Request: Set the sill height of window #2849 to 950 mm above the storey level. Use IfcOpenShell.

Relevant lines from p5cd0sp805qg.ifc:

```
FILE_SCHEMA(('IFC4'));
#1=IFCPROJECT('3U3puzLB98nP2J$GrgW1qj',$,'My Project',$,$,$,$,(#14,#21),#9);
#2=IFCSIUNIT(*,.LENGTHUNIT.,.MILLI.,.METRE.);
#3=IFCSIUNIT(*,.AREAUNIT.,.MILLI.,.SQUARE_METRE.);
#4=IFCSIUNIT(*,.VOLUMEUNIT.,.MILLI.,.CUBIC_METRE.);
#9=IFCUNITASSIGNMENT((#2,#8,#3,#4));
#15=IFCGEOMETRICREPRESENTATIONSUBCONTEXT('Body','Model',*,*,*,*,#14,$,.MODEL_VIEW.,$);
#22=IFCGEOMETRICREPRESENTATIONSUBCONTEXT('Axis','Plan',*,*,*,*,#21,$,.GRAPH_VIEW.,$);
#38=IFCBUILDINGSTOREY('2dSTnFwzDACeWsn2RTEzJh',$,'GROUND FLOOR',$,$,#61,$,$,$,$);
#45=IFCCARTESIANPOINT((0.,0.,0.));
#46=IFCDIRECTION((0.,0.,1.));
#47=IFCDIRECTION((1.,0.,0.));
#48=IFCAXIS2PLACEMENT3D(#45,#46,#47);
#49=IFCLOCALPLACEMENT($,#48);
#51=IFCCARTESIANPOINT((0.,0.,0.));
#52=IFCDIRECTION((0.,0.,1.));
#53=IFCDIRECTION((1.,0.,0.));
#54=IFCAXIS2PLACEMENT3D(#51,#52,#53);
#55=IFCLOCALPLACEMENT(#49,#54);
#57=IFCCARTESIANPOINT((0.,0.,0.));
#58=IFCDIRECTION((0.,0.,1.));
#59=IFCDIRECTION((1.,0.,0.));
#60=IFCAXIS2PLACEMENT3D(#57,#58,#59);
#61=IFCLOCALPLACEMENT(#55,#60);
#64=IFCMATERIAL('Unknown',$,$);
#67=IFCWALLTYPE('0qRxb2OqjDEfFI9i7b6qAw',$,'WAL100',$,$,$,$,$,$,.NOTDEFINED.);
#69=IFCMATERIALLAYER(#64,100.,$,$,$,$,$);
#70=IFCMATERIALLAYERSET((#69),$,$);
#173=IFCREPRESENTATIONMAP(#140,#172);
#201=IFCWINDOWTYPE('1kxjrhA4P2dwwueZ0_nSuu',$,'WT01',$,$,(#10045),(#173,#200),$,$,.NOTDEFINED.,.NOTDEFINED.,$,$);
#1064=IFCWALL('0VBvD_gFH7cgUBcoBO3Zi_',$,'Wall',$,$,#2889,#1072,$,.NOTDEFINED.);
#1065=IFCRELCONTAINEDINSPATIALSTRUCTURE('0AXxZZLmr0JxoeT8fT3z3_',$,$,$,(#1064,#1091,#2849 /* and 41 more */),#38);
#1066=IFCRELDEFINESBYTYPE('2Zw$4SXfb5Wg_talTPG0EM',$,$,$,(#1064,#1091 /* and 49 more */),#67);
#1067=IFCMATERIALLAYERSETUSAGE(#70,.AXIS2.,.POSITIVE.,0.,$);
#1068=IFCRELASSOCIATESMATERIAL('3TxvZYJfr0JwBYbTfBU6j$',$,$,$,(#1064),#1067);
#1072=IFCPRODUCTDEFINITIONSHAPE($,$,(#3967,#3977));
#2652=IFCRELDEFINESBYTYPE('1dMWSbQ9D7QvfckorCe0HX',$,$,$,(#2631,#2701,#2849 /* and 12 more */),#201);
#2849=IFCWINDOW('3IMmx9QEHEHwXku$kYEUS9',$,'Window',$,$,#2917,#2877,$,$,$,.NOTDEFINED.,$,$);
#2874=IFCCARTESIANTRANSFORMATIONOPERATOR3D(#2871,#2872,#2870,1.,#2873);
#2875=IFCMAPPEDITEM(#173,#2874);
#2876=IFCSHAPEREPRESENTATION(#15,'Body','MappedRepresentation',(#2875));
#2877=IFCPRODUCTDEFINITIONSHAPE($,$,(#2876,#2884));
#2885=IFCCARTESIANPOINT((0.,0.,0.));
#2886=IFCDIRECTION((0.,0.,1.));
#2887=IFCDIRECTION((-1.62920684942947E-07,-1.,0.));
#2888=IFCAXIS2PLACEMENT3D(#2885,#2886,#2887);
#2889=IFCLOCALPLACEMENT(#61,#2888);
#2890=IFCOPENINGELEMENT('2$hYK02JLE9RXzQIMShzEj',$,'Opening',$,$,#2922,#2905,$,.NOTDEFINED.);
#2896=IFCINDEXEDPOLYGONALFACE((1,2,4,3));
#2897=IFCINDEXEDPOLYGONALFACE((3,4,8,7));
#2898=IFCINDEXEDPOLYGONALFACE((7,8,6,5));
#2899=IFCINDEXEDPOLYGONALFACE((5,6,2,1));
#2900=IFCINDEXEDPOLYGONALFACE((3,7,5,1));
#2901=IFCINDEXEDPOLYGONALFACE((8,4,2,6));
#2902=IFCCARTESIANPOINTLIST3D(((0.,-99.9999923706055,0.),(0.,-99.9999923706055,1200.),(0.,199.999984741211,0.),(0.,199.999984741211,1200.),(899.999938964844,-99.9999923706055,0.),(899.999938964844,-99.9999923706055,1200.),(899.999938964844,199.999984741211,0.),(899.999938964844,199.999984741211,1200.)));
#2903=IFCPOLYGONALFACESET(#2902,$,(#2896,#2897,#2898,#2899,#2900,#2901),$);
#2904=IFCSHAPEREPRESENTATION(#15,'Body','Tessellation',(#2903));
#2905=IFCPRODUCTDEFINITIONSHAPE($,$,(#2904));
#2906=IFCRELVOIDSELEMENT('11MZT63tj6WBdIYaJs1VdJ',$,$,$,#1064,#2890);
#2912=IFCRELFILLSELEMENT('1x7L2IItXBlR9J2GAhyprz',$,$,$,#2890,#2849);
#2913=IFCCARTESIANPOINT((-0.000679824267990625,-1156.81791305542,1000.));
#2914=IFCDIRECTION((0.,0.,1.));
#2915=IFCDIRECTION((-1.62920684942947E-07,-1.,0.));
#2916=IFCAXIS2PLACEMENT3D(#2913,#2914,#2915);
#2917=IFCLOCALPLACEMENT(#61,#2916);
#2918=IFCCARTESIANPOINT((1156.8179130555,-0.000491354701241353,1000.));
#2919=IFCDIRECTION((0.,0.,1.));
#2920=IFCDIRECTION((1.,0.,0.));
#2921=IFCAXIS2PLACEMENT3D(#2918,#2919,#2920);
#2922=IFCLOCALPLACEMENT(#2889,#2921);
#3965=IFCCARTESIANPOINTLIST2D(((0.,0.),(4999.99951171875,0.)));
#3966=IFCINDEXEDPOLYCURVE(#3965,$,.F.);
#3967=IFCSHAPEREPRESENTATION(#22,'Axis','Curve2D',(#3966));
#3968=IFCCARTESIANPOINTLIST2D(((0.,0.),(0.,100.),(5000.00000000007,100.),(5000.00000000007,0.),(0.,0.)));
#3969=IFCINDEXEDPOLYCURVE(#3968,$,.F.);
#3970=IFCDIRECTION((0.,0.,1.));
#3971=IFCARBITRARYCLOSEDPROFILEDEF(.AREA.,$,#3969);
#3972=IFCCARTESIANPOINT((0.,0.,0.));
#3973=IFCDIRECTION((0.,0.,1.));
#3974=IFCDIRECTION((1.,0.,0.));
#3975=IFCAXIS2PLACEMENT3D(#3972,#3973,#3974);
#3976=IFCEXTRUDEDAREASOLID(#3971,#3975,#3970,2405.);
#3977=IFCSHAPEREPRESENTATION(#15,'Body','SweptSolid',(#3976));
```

```python
import numpy as np
import ifcopenshell
import ifcopenshell.api.geometry
import ifcopenshell.geom
import ifcopenshell.util.element
import ifcopenshell.util.placement
import ifcopenshell.util.shape
import ifcopenshell.util.unit

model = ifcopenshell.open("p5cd0sp805qg.ifc")
unit_scale = ifcopenshell.util.unit.calculate_unit_scale(model)

window = model.by_id(2849)
opening = window.FillsVoids[0].RelatingOpeningElement
storey = ifcopenshell.util.element.get_container(window, ifc_class="IfcBuildingStorey")
level = ifcopenshell.util.placement.get_local_placement(storey.ObjectPlacement)[2, 3]

# The opening's origin need not be at the sill, so measure its lowest point.
shape = ifcopenshell.geom.create_shape(ifcopenshell.geom.settings(), opening)
bottom = ifcopenshell.util.shape.get_shape_bottom_elevation(shape, shape.geometry) / unit_scale
dz = level + 0.95 / unit_scale - bottom

shift = np.array([0.0, 0.0, dz])
# The window is not placed relative to its opening, so move both.
for product in (opening, window):
    matrix = ifcopenshell.util.placement.get_local_placement(product.ObjectPlacement)
    matrix[:3, 3] += shift
    ifcopenshell.api.geometry.edit_object_placement(model, product=product, matrix=matrix, is_si=False)

print(f"moved by {dz * unit_scale:+.3f} m")

model.write("p5cd0sp805qg_rev.ifc")
```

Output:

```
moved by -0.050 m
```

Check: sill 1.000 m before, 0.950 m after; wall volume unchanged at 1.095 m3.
